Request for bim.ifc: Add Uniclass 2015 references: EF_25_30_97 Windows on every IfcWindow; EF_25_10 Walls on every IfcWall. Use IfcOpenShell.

First a look at what the model holds.

```python
import ifcopenshell

model = ifcopenshell.open("bim.ifc")
print(model.schema)
print("classifications:", [c.Name for c in model.by_type("IfcClassification")])
for ifc_class in ("IfcDoor", "IfcRoof", "IfcStair", "IfcWall", "IfcWindow"):
    print(ifc_class, len(model.by_type(ifc_class)))
```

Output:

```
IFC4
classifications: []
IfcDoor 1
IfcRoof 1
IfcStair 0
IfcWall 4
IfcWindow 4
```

```python
import ifcopenshell
import ifcopenshell.api.classification

model = ifcopenshell.open("bim.ifc")

system = ifcopenshell.api.classification.add_classification(model, classification="Uniclass 2015")

codes = {
    "IfcWindow": ("EF_25_30_97", "Windows"),
    "IfcWall": ("EF_25_10", "Walls"),
}
for ifc_class, (code, name) in codes.items():
    products = model.by_type(ifc_class)
    ifcopenshell.api.classification.add_reference(
        model, products=products, classification=system, identification=code, name=name
    )
    print(code, len(products))

model.write("bim_edited.ifc")
```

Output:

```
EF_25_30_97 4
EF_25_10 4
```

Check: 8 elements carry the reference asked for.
